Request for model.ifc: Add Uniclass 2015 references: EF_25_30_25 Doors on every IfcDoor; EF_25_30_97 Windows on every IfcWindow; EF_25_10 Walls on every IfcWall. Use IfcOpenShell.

First a look at what the model holds.

```python
import ifcopenshell

model = ifcopenshell.open("model.ifc")
print(model.schema)
print("classifications:", [c.Name for c in model.by_type("IfcClassification")])
for ifc_class in ("IfcDoor", "IfcRoof", "IfcStair", "IfcWall", "IfcWindow"):
    print(ifc_class, len(model.by_type(ifc_class)))
```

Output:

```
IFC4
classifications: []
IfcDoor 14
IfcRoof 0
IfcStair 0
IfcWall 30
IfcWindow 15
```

```python
import ifcopenshell
import ifcopenshell.api.classification

model = ifcopenshell.open("model.ifc")

system = ifcopenshell.api.classification.add_classification(model, classification="Uniclass 2015")

codes = {
    "IfcDoor": ("EF_25_30_25", "Doors"),
    "IfcWindow": ("EF_25_30_97", "Windows"),
    "IfcWall": ("EF_25_10", "Walls"),
}
for ifc_class, (code, name) in codes.items():
    products = model.by_type(ifc_class)
    ifcopenshell.api.classification.add_reference(
        model, products=products, classification=system, identification=code, name=name
    )
    print(code, len(products))

model.write("model_edited.ifc")
```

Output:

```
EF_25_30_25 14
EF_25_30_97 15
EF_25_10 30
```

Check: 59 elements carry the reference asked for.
